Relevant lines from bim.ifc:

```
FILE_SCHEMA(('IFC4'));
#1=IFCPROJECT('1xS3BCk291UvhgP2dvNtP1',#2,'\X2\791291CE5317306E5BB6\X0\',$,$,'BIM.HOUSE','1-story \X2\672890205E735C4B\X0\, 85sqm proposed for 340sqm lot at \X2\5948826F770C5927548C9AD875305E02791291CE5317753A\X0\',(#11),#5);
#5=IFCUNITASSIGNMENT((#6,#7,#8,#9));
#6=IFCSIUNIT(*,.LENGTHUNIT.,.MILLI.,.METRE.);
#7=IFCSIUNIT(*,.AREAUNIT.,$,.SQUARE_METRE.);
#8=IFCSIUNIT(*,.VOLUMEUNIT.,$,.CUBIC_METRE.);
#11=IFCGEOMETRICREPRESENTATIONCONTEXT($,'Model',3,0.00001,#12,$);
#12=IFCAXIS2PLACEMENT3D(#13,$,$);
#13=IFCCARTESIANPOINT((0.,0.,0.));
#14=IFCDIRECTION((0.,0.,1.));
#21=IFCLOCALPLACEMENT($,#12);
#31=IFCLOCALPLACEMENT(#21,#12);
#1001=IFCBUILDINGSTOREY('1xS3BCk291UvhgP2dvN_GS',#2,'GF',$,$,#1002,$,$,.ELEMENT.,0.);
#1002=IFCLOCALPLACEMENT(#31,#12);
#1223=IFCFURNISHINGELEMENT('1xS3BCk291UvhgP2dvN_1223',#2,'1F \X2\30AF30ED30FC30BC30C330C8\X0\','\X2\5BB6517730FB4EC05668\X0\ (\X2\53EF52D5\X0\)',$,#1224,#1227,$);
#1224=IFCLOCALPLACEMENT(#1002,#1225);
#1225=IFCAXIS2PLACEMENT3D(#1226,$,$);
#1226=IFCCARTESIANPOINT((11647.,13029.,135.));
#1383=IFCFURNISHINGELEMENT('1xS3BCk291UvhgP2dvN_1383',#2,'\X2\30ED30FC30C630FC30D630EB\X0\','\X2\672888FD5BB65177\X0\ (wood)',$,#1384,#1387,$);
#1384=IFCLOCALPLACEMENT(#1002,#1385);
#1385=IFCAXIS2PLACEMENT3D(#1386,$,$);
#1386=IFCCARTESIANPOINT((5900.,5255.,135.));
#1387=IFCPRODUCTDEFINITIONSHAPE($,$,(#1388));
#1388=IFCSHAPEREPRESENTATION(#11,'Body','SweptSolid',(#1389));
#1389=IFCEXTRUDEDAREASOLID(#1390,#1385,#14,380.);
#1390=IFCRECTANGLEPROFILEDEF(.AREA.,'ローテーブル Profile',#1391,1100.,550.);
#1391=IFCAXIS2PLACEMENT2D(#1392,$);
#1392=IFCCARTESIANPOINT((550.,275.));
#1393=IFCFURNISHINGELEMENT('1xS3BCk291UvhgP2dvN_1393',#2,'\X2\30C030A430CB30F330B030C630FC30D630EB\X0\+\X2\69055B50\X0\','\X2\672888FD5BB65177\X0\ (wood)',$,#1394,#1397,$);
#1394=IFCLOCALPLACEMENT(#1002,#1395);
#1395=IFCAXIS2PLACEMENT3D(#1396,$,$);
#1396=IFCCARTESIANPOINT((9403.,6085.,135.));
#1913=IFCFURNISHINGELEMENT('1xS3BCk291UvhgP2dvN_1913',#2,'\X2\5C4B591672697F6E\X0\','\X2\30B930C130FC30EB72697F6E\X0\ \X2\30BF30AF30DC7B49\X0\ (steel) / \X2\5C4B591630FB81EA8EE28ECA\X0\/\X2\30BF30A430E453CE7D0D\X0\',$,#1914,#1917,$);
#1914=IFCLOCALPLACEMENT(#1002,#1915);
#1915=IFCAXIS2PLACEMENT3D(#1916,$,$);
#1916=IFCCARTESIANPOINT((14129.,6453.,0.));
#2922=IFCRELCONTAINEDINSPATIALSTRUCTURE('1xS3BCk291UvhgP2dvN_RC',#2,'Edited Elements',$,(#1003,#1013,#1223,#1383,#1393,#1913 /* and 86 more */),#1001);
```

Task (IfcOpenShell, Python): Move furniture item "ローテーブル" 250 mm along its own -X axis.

```python
import ifcopenshell
import ifcopenshell.api.geometry
import ifcopenshell.util.placement
import ifcopenshell.util.unit

model = ifcopenshell.open("bim.ifc")
unit_scale = ifcopenshell.util.unit.calculate_unit_scale(model)

item = model.by_guid("1xS3BCk291UvhgP2dvN_1383")
matrix = ifcopenshell.util.placement.get_local_placement(item.ObjectPlacement)
matrix[:3, 3] -= matrix[:3, 0] * 0.25 / unit_scale
ifcopenshell.api.geometry.edit_object_placement(model, product=item, matrix=matrix, is_si=False)

print(ifcopenshell.util.placement.get_local_placement(item.ObjectPlacement).round(3) + 0.0)

model.write("bim_rev.ifc")
```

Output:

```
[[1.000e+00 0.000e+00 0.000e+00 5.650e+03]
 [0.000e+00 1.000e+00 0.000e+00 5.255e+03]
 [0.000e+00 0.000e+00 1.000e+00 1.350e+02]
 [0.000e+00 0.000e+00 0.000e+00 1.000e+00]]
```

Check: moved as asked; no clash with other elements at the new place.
